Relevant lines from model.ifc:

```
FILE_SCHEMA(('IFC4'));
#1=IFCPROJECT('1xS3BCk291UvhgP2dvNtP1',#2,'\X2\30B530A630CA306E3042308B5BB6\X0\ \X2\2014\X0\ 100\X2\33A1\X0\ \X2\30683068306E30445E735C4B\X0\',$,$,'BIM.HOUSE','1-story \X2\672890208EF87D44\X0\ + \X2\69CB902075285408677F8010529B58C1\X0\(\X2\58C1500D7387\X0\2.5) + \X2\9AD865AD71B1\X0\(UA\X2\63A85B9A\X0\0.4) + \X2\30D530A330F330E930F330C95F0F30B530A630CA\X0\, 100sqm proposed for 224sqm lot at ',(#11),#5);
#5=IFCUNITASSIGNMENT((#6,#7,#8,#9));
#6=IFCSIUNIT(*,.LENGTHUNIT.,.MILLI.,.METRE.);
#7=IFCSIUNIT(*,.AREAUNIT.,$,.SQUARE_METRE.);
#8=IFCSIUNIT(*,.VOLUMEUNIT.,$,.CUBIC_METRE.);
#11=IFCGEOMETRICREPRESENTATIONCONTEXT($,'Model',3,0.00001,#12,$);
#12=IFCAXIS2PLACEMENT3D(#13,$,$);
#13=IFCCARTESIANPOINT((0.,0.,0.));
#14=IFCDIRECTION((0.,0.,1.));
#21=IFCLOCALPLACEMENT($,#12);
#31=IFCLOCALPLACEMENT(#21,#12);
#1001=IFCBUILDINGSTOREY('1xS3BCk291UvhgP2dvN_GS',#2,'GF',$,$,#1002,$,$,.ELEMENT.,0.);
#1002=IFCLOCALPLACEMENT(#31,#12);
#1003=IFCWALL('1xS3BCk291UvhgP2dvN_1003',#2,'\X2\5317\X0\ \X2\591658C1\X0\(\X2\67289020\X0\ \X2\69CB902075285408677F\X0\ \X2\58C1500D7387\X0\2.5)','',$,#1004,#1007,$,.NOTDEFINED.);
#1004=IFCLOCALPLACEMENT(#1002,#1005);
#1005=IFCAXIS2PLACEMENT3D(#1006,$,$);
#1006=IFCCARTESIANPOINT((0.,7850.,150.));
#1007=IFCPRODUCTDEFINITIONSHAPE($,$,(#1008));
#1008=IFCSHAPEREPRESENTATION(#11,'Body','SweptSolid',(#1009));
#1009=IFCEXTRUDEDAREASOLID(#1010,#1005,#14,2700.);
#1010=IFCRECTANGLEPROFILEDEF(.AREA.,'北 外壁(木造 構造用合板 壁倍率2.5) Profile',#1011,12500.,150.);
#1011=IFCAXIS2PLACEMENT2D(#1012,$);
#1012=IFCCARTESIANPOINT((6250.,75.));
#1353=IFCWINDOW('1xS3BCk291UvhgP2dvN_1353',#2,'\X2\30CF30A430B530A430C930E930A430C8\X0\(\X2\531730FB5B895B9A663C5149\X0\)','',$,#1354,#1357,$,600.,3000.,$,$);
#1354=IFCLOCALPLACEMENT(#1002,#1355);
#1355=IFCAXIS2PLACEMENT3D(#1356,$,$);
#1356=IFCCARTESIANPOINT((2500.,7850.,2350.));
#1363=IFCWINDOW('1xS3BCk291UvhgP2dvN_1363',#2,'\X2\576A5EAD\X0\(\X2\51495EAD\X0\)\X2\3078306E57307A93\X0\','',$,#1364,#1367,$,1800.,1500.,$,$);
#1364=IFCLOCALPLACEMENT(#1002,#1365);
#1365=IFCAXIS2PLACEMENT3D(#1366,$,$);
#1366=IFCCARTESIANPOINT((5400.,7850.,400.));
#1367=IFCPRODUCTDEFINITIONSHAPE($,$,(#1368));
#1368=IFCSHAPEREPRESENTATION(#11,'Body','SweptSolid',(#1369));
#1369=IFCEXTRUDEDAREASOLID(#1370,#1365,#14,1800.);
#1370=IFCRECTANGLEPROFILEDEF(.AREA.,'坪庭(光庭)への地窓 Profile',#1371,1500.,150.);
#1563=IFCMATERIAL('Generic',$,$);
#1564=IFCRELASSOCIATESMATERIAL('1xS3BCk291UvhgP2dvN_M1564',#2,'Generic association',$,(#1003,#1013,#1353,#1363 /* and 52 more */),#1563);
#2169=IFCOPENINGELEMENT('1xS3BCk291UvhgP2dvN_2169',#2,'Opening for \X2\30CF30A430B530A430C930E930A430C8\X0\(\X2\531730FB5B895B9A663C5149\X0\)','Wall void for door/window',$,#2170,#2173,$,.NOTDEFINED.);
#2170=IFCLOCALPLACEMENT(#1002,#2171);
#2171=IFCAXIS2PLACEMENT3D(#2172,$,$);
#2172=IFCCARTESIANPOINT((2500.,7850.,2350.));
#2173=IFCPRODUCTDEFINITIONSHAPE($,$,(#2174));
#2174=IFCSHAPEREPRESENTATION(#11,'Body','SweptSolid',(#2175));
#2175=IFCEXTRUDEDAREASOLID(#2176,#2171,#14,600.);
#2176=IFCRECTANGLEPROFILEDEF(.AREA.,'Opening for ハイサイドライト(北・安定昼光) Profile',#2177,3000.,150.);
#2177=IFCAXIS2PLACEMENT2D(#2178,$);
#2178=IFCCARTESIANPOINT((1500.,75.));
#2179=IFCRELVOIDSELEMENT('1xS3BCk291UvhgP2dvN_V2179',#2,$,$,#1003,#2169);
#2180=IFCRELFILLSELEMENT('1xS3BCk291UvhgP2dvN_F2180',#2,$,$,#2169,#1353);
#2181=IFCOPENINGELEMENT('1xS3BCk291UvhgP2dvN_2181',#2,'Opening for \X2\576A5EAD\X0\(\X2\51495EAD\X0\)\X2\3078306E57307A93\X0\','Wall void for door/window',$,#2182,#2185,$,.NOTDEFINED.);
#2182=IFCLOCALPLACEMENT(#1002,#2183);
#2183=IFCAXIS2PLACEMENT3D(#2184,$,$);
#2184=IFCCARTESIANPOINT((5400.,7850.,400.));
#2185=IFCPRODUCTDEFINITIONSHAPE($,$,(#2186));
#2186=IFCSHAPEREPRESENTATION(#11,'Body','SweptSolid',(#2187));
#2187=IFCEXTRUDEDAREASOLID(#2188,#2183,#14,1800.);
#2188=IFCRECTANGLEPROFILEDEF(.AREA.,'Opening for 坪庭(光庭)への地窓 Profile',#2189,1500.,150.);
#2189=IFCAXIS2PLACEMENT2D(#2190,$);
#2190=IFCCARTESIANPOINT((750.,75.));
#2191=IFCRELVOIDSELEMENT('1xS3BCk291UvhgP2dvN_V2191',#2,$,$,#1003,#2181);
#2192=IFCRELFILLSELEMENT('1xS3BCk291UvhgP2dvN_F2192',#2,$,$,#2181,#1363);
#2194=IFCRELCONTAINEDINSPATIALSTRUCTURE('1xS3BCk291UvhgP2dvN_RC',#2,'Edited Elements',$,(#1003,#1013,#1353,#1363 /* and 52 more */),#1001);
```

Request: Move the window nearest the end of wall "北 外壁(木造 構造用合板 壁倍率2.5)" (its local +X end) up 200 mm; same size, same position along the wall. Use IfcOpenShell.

```python
import numpy as np
import ifcopenshell
import ifcopenshell.api.geometry
import ifcopenshell.util.placement
import ifcopenshell.util.unit

model = ifcopenshell.open("model.ifc")
unit_scale = ifcopenshell.util.unit.calculate_unit_scale(model)

window = model.by_guid("1xS3BCk291UvhgP2dvN_1363")
opening = window.FillsVoids[0].RelatingOpeningElement
dz = 0.2 / unit_scale

shift = np.array([0.0, 0.0, dz])
# The window is not placed relative to its opening, so move both.
for product in (opening, window):
    matrix = ifcopenshell.util.placement.get_local_placement(product.ObjectPlacement)
    matrix[:3, 3] += shift
    ifcopenshell.api.geometry.edit_object_placement(model, product=product, matrix=matrix, is_si=False)

print(f"moved by {dz * unit_scale:+.3f} m")

model.write("model_rev.ifc")
```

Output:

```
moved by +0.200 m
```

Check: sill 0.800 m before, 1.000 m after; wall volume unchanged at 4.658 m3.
